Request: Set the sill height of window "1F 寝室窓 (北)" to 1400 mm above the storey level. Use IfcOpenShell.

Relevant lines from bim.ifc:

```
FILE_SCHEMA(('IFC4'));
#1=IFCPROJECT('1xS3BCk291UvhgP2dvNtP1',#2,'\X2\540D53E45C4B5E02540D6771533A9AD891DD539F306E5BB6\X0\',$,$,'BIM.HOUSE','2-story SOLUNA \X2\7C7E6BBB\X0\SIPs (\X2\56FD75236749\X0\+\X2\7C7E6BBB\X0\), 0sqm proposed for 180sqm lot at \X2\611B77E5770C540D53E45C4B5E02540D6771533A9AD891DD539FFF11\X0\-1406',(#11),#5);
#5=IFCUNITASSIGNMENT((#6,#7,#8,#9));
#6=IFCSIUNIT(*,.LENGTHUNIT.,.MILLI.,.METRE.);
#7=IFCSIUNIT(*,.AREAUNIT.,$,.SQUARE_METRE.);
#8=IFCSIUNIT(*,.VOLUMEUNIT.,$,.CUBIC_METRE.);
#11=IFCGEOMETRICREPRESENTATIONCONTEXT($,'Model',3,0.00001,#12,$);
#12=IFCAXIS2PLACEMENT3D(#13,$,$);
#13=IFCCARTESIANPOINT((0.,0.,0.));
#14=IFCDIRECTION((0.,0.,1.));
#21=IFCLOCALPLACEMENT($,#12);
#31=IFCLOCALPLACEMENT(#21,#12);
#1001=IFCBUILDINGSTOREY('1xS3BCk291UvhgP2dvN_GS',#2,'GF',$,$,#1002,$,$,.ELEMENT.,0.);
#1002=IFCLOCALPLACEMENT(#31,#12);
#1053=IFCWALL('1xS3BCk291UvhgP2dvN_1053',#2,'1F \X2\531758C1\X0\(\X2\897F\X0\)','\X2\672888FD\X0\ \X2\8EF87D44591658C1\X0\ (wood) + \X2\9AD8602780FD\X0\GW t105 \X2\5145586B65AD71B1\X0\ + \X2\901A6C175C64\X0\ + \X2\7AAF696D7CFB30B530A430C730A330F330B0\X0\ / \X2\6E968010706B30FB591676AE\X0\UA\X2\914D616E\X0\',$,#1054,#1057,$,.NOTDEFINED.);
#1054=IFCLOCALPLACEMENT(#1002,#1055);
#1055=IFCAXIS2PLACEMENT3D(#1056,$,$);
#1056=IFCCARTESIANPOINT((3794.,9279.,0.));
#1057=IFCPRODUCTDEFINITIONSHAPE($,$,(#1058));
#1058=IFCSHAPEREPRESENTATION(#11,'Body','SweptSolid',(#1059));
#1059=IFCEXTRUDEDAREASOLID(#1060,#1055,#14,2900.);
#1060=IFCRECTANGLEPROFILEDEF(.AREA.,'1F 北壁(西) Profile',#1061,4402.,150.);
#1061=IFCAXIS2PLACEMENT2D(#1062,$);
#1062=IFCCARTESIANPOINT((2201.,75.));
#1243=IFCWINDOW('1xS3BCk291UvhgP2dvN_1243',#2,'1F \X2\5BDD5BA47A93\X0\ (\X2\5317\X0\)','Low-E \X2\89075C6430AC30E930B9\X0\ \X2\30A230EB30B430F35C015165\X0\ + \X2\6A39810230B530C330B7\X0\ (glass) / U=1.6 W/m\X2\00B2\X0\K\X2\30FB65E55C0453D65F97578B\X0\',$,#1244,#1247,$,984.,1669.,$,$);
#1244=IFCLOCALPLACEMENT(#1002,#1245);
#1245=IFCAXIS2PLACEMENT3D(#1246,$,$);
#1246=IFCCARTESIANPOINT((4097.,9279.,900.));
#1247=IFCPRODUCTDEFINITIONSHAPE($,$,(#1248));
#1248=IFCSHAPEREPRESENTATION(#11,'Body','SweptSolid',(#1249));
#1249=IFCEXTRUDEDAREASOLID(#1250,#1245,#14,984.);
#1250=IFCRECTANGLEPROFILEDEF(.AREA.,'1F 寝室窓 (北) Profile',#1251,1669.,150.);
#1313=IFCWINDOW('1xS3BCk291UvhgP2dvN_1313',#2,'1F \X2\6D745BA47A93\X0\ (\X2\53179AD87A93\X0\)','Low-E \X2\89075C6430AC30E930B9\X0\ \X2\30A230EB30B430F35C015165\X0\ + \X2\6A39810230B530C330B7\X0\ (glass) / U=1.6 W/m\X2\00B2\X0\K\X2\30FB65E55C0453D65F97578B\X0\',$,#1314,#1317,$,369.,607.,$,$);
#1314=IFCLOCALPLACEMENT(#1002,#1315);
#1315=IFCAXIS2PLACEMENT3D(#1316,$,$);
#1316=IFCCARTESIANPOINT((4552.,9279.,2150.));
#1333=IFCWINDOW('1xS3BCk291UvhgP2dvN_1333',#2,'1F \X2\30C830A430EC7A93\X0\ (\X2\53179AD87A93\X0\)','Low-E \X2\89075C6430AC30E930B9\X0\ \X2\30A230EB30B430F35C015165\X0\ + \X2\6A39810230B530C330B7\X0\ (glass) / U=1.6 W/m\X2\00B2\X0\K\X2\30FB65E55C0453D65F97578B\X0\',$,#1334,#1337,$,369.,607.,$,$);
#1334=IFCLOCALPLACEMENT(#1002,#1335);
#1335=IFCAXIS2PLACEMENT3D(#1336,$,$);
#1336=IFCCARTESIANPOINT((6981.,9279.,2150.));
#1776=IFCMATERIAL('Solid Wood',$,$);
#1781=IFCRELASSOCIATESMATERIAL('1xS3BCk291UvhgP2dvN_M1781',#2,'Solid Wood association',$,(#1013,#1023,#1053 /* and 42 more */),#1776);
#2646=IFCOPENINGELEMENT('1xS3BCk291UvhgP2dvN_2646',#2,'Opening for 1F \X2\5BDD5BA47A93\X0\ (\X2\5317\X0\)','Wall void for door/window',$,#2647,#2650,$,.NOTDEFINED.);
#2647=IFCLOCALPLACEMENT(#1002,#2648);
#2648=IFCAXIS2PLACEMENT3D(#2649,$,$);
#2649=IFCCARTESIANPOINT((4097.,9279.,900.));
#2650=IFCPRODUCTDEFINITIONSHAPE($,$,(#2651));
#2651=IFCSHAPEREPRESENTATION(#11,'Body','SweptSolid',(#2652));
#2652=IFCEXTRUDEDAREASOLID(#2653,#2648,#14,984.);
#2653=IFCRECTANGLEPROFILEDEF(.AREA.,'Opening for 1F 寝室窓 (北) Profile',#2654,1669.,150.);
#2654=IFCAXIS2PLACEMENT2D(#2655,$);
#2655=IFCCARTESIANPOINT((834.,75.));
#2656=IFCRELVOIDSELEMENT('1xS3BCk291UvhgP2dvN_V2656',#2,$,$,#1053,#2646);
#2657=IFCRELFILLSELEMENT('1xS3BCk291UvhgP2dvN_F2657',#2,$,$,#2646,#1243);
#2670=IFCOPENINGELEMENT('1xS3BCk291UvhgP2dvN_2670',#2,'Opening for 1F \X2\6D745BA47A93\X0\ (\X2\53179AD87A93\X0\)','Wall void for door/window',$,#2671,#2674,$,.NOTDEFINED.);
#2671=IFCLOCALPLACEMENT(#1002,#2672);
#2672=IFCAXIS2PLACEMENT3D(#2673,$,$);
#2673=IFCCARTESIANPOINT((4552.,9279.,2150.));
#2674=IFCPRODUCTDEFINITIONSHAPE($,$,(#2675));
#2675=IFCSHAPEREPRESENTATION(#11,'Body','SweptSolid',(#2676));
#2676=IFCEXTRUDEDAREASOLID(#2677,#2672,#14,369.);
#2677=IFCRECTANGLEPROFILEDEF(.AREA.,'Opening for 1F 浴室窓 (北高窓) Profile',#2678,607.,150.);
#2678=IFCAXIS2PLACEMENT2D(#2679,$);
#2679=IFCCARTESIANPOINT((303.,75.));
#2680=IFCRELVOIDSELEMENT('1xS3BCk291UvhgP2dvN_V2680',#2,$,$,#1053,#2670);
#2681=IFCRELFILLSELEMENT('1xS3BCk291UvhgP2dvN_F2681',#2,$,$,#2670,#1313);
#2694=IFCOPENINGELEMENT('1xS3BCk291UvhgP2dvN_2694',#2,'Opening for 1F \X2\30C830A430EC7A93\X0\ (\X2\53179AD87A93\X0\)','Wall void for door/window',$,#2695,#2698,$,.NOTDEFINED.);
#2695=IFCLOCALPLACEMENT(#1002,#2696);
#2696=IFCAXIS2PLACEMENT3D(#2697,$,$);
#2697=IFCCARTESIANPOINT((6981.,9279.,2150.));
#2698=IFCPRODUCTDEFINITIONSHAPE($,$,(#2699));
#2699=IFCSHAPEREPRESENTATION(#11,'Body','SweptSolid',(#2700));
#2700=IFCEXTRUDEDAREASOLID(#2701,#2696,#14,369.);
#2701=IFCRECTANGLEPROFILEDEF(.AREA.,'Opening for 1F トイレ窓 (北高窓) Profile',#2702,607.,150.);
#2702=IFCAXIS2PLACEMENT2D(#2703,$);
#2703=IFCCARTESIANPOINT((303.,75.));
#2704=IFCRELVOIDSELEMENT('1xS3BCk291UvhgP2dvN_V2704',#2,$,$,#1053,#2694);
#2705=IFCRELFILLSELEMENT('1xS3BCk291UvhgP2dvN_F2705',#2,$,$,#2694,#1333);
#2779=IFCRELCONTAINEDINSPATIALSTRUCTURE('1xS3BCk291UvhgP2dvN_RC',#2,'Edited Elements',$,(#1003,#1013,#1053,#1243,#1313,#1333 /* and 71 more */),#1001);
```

```python
import numpy as np
import ifcopenshell
import ifcopenshell.api.geometry
import ifcopenshell.geom
import ifcopenshell.util.element
import ifcopenshell.util.placement
import ifcopenshell.util.shape
import ifcopenshell.util.unit

model = ifcopenshell.open("bim.ifc")
unit_scale = ifcopenshell.util.unit.calculate_unit_scale(model)

window = model.by_id(1243)
opening = window.FillsVoids[0].RelatingOpeningElement
storey = ifcopenshell.util.element.get_container(window, ifc_class="IfcBuildingStorey")
level = ifcopenshell.util.placement.get_local_placement(storey.ObjectPlacement)[2, 3]

# The opening's origin need not be at the sill, so measure its lowest point.
shape = ifcopenshell.geom.create_shape(ifcopenshell.geom.settings(), opening)
bottom = ifcopenshell.util.shape.get_shape_bottom_elevation(shape, shape.geometry) / unit_scale
dz = level + 1400.0 - bottom

shift = np.array([0.0, 0.0, dz])
# The window is not placed relative to its opening, so move both.
for product in (opening, window):
    matrix = ifcopenshell.util.placement.get_local_placement(product.ObjectPlacement)
    matrix[:3, 3] += shift
    ifcopenshell.api.geometry.edit_object_placement(model, product=product, matrix=matrix, is_si=False)

print(f"moved by {dz * unit_scale:+.3f} m")

model.write("bim_rev.ifc")
```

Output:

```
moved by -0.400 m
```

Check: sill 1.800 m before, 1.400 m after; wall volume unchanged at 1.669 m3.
